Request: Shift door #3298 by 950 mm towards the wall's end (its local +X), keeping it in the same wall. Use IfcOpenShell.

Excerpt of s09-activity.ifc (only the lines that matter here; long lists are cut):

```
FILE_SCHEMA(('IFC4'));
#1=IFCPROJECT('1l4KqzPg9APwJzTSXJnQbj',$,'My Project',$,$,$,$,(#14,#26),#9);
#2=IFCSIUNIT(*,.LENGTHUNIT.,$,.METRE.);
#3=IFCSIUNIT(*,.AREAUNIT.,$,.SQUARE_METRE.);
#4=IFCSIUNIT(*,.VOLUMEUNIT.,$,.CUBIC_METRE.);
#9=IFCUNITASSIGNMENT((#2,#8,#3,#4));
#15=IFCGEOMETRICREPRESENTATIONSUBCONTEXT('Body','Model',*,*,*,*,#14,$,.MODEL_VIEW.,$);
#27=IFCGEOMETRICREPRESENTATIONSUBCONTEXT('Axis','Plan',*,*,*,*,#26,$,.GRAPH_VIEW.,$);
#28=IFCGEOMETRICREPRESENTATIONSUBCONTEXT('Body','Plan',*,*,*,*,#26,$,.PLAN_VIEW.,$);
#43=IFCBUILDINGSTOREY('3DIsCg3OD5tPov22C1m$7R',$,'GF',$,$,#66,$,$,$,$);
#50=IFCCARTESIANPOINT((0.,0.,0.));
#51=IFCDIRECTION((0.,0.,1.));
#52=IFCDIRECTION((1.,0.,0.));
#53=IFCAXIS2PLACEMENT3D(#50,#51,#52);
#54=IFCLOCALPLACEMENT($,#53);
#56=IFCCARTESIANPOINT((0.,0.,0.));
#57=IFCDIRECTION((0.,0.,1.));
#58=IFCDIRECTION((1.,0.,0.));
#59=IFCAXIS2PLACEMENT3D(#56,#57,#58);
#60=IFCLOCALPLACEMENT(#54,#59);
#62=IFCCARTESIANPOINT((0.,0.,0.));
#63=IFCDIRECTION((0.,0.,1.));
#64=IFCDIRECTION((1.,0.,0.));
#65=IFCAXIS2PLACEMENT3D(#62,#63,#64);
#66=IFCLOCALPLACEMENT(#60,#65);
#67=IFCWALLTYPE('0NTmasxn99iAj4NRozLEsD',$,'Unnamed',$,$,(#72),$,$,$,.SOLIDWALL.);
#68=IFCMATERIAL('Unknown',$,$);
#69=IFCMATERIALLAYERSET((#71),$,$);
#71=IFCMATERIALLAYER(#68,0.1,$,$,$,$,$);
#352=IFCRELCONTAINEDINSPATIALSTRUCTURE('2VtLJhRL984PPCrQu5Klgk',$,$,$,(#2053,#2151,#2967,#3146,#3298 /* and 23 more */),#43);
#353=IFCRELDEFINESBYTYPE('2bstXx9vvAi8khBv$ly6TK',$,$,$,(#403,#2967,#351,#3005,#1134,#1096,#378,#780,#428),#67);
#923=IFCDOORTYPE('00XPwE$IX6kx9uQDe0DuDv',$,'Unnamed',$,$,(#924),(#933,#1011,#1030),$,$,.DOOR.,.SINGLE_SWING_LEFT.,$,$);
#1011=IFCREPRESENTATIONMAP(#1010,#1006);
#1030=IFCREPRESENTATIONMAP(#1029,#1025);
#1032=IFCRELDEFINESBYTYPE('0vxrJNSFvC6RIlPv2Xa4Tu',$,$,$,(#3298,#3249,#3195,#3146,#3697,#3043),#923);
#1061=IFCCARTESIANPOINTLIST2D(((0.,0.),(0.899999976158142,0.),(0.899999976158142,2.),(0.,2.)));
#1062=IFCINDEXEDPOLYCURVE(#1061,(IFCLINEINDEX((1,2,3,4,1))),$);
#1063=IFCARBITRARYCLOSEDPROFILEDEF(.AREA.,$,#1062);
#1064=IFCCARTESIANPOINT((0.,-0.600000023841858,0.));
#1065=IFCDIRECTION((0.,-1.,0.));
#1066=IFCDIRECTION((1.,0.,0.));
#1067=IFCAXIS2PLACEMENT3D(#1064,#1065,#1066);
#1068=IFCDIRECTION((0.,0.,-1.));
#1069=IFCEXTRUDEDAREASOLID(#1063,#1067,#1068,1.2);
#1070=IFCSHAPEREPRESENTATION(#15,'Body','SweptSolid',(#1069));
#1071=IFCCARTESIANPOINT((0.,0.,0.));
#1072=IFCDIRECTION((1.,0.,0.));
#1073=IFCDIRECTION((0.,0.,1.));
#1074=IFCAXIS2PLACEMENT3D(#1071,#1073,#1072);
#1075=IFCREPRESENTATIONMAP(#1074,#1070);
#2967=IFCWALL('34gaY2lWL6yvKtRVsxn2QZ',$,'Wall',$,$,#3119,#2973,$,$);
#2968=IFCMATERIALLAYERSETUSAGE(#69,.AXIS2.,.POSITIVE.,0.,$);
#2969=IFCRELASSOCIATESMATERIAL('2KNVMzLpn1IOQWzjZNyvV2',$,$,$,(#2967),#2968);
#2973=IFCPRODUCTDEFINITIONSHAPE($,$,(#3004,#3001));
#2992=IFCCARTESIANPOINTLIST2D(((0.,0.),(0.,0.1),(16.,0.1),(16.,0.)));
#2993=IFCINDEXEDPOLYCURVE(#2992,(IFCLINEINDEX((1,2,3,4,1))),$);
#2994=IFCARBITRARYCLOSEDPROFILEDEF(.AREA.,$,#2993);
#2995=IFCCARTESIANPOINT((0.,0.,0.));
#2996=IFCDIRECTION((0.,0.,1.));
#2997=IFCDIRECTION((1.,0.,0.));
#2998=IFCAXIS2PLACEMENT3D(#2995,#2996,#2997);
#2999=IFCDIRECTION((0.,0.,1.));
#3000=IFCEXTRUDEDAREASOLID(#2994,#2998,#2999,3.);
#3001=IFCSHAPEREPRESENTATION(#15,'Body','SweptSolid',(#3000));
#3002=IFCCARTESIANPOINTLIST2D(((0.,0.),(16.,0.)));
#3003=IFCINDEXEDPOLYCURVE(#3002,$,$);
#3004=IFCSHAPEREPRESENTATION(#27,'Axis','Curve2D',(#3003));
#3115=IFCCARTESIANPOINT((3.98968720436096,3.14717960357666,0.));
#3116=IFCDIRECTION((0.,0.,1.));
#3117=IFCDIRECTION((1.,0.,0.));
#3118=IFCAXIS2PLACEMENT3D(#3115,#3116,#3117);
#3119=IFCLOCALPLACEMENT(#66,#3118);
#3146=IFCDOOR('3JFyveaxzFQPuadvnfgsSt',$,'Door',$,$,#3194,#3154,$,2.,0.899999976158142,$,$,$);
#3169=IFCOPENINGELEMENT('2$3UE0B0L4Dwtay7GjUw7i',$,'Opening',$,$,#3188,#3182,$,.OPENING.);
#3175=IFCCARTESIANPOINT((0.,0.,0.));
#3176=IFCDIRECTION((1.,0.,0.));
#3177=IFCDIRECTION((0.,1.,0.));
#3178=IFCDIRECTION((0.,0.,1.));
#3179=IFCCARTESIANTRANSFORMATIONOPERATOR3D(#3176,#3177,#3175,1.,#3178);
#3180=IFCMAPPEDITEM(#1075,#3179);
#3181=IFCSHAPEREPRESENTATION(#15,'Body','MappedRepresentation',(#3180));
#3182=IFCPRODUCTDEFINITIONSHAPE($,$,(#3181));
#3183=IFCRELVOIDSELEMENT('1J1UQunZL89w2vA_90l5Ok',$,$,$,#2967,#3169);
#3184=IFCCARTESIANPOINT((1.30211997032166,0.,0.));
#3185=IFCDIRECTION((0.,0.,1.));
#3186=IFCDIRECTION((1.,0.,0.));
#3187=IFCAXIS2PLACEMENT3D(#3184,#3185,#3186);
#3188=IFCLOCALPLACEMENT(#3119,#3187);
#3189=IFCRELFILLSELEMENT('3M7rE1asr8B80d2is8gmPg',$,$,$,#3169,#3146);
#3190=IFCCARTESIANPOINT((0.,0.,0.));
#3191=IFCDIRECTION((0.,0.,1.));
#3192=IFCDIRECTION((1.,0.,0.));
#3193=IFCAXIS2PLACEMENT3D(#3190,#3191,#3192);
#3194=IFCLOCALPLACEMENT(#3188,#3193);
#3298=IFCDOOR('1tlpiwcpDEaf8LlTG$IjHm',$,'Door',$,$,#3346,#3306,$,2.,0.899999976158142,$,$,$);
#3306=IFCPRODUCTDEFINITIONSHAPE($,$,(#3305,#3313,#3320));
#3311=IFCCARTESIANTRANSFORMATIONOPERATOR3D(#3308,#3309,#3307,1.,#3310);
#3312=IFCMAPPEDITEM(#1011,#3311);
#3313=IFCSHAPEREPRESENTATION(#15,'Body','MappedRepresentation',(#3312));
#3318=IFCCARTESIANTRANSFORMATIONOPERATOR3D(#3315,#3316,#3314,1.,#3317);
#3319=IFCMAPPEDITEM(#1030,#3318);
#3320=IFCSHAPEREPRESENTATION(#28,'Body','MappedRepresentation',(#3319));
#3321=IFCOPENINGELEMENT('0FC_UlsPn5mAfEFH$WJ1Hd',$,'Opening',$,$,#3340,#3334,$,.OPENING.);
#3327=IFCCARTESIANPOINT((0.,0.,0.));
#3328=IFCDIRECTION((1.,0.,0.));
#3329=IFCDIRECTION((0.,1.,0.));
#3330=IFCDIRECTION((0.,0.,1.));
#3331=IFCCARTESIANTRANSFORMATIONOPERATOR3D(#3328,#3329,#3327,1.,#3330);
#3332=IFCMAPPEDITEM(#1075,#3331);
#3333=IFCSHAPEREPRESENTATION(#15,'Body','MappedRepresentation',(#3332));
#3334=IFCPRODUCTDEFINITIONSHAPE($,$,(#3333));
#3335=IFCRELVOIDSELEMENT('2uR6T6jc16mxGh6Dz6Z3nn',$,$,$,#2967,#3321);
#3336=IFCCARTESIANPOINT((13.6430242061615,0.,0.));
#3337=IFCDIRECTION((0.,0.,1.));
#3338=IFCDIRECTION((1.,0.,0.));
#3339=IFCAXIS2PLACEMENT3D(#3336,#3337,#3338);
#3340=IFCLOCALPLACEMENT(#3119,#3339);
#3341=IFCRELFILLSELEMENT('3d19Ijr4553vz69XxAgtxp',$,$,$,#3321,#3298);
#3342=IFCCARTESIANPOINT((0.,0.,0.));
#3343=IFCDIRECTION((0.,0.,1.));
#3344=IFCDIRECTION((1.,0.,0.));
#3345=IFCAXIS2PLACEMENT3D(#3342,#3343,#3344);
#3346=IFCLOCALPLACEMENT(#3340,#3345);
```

```python
import ifcopenshell
import ifcopenshell.api.geometry
import ifcopenshell.util.placement
import ifcopenshell.util.unit

model = ifcopenshell.open("s09-activity.ifc")
unit_scale = ifcopenshell.util.unit.calculate_unit_scale(model)

door = model.by_guid("1tlpiwcpDEaf8LlTG$IjHm")
opening = door.FillsVoids[0].RelatingOpeningElement
wall = opening.VoidsElements[0].RelatingBuildingElement

wall_matrix = ifcopenshell.util.placement.get_local_placement(wall.ObjectPlacement)
shift = wall_matrix[:3, 0] * 0.95 / unit_scale
before = ifcopenshell.util.placement.get_local_placement(door.ObjectPlacement)[:3, 3].copy()

# The door is placed relative to its opening, so it follows when the opening moves.
matrix = ifcopenshell.util.placement.get_local_placement(opening.ObjectPlacement)
matrix[:3, 3] += shift
ifcopenshell.api.geometry.edit_object_placement(
    model, product=opening, matrix=matrix, is_si=False, should_transform_children=True
)

after = ifcopenshell.util.placement.get_local_placement(door.ObjectPlacement)[:3, 3]
print("door moved by", (after - before).round(3) + 0.0)

model.write("s09-activity_rev.ifc")
```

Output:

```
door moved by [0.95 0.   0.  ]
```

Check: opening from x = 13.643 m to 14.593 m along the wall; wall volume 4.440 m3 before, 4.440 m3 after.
